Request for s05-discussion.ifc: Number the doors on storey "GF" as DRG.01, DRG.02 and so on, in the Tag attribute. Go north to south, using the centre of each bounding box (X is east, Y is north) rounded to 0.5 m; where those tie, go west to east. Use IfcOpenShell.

First a look at what the model holds.

```python
import ifcopenshell
import ifcopenshell.util.element
import ifcopenshell.util.placement

model = ifcopenshell.open("s05-discussion.ifc")
print(model.schema)
storey = next(s for s in model.by_type("IfcBuildingStorey") if s.Name == "GF")
doors = [e for e in ifcopenshell.util.element.get_decomposition(storey) if e.is_a("IfcDoor")]
for e in sorted(doors, key=lambda e: e.id()):
    origin = ifcopenshell.util.placement.get_local_placement(e.ObjectPlacement)[:3, 3]
    print(e.id(), e.Tag, e.Name, origin.round(2) + 0.0, sep=" | ")
```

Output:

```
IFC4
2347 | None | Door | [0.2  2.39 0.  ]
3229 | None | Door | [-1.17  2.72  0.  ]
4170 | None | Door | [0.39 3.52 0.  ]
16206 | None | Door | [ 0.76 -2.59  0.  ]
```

```python
import ifcopenshell
import ifcopenshell.geom
import ifcopenshell.util.element
import ifcopenshell.util.shape

model = ifcopenshell.open("s05-discussion.ifc")
settings = ifcopenshell.geom.settings()
settings.set("use-world-coords", True)


def centre(element):
    shape = ifcopenshell.geom.create_shape(settings, element)
    return ifcopenshell.util.shape.get_bbox_centroid(shape.geometry)


storey = next(s for s in model.by_type("IfcBuildingStorey") if s.Name == "GF")
doors = [e for e in ifcopenshell.util.element.get_decomposition(storey) if e.is_a("IfcDoor")]

# Insertion points can sit at a corner or the storey origin, so sort by the geometry (in metres).
centres = {e: centre(e) for e in doors}
doors.sort(key=lambda e: (-round(centres[e][1] / 0.5), centres[e][0]))

for i, e in enumerate(doors, start=1):
    number = f"DRG.{i:02d}"
    e.Tag = number
    print(e.id(), number)

model.write("s05-discussion_edited.ifc")
```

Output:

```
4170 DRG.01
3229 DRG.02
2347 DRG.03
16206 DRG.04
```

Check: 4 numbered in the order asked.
